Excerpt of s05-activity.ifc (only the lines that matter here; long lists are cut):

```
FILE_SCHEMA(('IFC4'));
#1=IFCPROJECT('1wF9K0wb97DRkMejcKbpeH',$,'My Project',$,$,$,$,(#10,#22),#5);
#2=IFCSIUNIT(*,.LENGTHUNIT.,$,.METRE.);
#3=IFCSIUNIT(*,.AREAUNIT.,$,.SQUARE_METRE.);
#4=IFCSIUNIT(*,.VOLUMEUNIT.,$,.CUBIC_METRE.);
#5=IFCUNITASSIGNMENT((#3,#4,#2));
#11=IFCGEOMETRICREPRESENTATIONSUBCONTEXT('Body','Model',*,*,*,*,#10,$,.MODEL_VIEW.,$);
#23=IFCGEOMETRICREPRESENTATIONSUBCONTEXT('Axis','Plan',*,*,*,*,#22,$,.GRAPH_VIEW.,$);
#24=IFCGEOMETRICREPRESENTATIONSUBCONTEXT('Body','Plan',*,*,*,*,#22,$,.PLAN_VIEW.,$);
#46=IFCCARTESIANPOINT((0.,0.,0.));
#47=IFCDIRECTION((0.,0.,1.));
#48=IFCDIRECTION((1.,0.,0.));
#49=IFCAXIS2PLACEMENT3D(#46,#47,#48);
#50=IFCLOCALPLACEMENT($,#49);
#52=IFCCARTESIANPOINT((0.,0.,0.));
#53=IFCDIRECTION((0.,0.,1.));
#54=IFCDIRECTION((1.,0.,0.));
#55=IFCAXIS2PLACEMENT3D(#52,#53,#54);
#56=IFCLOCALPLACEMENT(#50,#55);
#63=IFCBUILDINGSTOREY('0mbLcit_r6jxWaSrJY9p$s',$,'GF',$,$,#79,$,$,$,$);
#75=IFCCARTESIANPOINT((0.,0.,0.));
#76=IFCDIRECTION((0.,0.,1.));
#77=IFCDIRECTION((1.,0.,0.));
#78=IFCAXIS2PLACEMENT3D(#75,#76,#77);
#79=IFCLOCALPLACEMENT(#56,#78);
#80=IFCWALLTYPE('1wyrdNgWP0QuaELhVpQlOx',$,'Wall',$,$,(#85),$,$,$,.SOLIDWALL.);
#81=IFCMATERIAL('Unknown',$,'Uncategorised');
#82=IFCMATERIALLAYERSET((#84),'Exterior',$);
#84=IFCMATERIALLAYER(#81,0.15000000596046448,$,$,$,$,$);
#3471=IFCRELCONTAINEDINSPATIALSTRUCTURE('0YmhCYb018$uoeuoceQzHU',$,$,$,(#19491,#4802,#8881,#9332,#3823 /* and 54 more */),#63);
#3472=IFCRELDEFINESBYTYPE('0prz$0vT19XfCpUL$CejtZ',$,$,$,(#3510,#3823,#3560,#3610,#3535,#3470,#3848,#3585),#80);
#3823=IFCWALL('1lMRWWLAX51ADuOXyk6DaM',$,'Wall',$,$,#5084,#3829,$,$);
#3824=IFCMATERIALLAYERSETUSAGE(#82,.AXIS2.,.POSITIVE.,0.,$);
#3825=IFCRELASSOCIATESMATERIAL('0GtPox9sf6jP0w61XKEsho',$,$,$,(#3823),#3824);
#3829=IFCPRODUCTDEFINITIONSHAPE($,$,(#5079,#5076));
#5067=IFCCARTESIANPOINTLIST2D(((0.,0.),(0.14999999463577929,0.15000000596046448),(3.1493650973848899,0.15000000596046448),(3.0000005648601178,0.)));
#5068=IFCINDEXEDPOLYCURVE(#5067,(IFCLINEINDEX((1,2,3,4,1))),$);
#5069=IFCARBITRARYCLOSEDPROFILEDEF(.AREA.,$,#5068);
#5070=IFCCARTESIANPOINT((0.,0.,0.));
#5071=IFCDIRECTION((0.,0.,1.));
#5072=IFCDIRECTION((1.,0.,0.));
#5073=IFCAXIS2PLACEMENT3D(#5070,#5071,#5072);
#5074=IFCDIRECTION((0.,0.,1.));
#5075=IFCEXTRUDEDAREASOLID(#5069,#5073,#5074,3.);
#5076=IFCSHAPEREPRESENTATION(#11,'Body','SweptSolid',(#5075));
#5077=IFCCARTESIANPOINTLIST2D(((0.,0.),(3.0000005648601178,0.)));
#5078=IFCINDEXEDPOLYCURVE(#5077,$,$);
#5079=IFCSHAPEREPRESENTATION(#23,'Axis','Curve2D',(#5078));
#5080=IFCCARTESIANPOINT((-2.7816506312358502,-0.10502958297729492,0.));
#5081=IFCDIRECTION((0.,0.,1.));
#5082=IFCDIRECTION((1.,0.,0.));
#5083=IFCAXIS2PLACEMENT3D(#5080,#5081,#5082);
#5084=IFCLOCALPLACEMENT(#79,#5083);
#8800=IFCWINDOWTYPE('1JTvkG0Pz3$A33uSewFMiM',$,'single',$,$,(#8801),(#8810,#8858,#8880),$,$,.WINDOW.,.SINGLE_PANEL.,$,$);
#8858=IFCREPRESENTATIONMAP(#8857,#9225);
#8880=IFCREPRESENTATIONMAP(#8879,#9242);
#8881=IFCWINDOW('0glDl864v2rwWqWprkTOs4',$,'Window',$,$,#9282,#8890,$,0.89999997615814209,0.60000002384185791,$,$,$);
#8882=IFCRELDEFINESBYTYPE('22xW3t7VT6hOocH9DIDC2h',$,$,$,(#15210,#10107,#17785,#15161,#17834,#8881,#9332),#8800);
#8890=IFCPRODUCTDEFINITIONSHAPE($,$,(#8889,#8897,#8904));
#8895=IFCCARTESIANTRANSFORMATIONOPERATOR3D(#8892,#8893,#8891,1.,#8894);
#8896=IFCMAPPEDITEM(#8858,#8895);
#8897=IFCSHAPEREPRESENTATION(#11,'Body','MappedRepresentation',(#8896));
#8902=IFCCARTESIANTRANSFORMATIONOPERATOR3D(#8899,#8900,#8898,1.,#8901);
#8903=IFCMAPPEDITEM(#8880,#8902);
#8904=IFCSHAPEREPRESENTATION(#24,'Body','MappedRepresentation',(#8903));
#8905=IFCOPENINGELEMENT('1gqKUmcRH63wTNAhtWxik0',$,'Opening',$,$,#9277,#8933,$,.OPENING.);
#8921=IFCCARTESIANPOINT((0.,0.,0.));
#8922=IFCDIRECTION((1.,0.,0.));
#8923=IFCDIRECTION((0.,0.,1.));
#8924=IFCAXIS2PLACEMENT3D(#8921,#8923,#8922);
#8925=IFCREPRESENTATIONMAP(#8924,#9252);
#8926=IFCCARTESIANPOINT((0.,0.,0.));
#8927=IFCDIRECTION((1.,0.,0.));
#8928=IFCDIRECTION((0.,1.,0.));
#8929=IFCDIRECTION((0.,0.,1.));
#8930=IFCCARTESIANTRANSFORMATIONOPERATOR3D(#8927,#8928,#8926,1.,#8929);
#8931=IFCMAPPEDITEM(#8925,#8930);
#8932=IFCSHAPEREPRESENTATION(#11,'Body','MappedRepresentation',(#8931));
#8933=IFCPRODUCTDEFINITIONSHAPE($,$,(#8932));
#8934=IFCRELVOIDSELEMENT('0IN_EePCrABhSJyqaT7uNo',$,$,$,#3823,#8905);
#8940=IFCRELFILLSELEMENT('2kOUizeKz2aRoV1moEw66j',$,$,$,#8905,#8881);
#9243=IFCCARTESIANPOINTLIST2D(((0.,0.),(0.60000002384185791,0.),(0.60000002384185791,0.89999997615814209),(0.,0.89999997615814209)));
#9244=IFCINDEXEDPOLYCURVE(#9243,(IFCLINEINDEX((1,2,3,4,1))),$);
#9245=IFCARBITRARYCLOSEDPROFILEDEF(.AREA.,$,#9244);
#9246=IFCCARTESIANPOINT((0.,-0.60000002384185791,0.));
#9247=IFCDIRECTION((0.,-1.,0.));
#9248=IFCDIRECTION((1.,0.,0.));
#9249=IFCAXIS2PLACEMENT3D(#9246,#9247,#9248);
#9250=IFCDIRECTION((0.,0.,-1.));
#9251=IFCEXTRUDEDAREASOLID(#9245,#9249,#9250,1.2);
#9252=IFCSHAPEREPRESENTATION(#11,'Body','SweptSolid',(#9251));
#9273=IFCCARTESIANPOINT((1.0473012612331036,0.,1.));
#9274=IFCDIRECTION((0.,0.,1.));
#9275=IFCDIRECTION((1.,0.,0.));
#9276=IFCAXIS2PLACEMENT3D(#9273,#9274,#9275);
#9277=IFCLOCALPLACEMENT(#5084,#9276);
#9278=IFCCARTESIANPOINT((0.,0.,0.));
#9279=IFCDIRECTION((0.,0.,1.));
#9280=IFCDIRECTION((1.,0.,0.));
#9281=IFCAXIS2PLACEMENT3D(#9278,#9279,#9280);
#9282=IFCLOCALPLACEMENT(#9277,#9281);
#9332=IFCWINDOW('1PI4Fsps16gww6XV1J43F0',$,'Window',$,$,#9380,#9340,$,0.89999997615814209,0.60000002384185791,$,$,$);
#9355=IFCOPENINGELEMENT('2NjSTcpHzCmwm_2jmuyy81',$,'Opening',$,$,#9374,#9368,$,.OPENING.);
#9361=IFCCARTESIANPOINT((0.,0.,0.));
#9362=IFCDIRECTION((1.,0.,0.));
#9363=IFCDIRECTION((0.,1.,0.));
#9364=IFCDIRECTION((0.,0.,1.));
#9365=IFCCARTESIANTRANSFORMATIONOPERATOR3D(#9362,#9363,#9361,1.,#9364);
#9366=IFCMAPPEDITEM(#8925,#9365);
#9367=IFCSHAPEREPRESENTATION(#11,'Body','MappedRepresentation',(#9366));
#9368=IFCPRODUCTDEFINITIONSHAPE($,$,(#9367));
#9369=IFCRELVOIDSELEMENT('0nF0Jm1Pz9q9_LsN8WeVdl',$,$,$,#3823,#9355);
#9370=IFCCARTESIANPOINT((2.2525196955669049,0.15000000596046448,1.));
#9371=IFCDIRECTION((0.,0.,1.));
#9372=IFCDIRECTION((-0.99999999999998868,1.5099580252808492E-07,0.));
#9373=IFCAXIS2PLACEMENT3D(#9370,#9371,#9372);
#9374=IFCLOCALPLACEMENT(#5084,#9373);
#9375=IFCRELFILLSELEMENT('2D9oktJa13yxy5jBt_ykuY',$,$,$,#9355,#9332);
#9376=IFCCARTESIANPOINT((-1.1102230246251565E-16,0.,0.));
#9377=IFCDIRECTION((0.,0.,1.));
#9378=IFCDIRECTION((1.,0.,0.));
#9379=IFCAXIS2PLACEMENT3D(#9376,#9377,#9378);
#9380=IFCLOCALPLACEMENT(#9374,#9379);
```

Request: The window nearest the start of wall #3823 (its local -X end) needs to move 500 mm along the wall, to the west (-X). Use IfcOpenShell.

```python
import ifcopenshell
import ifcopenshell.api.geometry
import ifcopenshell.util.placement
import ifcopenshell.util.unit

model = ifcopenshell.open("s05-activity.ifc")
unit_scale = ifcopenshell.util.unit.calculate_unit_scale(model)

window = model.by_guid("0glDl864v2rwWqWprkTOs4")
opening = window.FillsVoids[0].RelatingOpeningElement
wall = opening.VoidsElements[0].RelatingBuildingElement

wall_matrix = ifcopenshell.util.placement.get_local_placement(wall.ObjectPlacement)
shift = wall_matrix[:3, 0] * -0.5 / unit_scale
before = ifcopenshell.util.placement.get_local_placement(window.ObjectPlacement)[:3, 3].copy()

# The window is placed relative to its opening, so it follows when the opening moves.
matrix = ifcopenshell.util.placement.get_local_placement(opening.ObjectPlacement)
matrix[:3, 3] += shift
ifcopenshell.api.geometry.edit_object_placement(
    model, product=opening, matrix=matrix, is_si=False, should_transform_children=True
)

after = ifcopenshell.util.placement.get_local_placement(window.ObjectPlacement)[:3, 3]
print("window moved by", (after - before).round(3) + 0.0)

model.write("s05-activity_updated.ifc")
```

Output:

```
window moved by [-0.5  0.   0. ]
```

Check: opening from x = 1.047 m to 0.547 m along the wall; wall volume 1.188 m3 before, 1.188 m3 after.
